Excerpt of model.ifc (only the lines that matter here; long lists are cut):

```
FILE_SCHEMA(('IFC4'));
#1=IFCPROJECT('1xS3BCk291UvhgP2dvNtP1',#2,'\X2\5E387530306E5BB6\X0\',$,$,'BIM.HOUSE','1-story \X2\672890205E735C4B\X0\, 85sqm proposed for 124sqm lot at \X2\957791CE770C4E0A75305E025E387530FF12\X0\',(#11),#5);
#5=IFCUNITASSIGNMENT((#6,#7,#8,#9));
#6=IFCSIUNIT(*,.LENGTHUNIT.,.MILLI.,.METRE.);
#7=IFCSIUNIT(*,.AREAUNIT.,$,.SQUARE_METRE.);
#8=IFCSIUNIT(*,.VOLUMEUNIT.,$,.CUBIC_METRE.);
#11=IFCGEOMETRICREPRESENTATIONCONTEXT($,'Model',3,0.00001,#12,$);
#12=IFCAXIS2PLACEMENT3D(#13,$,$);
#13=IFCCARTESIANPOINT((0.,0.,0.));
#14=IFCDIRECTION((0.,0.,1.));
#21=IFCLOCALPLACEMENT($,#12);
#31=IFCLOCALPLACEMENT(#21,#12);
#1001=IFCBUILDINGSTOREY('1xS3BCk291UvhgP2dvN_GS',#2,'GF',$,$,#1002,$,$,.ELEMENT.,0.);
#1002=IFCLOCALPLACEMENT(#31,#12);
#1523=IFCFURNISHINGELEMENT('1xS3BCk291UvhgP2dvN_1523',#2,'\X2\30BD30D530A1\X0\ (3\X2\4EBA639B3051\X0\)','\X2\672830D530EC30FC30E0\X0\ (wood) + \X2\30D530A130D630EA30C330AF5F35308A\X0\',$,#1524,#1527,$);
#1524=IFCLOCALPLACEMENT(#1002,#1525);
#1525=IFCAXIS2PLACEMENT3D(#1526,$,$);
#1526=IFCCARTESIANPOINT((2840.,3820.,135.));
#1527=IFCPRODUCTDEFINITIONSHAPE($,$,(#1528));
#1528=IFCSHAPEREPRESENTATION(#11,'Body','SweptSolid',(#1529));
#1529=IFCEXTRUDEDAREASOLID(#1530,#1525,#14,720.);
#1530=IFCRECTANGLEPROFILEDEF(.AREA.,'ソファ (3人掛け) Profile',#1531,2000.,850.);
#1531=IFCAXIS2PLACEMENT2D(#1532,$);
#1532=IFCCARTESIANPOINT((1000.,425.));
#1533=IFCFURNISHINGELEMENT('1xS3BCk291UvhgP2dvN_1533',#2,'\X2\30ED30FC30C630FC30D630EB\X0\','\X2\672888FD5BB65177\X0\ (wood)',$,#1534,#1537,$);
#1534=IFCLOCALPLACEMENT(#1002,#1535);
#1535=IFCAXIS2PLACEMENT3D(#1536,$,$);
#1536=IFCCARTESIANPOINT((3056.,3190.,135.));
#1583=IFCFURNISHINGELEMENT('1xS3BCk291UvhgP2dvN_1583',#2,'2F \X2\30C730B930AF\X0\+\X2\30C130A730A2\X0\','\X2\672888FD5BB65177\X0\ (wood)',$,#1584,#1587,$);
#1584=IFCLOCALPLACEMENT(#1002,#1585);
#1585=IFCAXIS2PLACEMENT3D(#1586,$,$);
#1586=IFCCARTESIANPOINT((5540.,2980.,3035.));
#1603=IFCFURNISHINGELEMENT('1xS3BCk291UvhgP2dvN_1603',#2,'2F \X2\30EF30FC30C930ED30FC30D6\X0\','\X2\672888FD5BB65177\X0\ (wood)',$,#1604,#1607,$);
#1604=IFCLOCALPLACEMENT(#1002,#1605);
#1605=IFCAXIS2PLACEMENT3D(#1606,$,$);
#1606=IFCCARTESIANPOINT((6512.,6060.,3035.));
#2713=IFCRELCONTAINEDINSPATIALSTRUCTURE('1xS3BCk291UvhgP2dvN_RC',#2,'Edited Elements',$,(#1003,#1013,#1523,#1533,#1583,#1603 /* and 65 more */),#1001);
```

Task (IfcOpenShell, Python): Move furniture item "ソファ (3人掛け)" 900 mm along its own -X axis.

```python
import ifcopenshell
import ifcopenshell.api.geometry
import ifcopenshell.util.placement
import ifcopenshell.util.unit

model = ifcopenshell.open("model.ifc")
unit_scale = ifcopenshell.util.unit.calculate_unit_scale(model)

item = model.by_guid("1xS3BCk291UvhgP2dvN_1523")
matrix = ifcopenshell.util.placement.get_local_placement(item.ObjectPlacement)
matrix[:3, 3] -= matrix[:3, 0] * 0.9 / unit_scale
ifcopenshell.api.geometry.edit_object_placement(model, product=item, matrix=matrix, is_si=False)

print(ifcopenshell.util.placement.get_local_placement(item.ObjectPlacement).round(3) + 0.0)

model.write("model_edited.ifc")
```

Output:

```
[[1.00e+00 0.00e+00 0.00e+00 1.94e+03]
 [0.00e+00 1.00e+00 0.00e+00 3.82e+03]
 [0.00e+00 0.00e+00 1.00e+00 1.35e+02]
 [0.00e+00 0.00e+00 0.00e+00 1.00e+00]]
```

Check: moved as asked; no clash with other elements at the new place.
